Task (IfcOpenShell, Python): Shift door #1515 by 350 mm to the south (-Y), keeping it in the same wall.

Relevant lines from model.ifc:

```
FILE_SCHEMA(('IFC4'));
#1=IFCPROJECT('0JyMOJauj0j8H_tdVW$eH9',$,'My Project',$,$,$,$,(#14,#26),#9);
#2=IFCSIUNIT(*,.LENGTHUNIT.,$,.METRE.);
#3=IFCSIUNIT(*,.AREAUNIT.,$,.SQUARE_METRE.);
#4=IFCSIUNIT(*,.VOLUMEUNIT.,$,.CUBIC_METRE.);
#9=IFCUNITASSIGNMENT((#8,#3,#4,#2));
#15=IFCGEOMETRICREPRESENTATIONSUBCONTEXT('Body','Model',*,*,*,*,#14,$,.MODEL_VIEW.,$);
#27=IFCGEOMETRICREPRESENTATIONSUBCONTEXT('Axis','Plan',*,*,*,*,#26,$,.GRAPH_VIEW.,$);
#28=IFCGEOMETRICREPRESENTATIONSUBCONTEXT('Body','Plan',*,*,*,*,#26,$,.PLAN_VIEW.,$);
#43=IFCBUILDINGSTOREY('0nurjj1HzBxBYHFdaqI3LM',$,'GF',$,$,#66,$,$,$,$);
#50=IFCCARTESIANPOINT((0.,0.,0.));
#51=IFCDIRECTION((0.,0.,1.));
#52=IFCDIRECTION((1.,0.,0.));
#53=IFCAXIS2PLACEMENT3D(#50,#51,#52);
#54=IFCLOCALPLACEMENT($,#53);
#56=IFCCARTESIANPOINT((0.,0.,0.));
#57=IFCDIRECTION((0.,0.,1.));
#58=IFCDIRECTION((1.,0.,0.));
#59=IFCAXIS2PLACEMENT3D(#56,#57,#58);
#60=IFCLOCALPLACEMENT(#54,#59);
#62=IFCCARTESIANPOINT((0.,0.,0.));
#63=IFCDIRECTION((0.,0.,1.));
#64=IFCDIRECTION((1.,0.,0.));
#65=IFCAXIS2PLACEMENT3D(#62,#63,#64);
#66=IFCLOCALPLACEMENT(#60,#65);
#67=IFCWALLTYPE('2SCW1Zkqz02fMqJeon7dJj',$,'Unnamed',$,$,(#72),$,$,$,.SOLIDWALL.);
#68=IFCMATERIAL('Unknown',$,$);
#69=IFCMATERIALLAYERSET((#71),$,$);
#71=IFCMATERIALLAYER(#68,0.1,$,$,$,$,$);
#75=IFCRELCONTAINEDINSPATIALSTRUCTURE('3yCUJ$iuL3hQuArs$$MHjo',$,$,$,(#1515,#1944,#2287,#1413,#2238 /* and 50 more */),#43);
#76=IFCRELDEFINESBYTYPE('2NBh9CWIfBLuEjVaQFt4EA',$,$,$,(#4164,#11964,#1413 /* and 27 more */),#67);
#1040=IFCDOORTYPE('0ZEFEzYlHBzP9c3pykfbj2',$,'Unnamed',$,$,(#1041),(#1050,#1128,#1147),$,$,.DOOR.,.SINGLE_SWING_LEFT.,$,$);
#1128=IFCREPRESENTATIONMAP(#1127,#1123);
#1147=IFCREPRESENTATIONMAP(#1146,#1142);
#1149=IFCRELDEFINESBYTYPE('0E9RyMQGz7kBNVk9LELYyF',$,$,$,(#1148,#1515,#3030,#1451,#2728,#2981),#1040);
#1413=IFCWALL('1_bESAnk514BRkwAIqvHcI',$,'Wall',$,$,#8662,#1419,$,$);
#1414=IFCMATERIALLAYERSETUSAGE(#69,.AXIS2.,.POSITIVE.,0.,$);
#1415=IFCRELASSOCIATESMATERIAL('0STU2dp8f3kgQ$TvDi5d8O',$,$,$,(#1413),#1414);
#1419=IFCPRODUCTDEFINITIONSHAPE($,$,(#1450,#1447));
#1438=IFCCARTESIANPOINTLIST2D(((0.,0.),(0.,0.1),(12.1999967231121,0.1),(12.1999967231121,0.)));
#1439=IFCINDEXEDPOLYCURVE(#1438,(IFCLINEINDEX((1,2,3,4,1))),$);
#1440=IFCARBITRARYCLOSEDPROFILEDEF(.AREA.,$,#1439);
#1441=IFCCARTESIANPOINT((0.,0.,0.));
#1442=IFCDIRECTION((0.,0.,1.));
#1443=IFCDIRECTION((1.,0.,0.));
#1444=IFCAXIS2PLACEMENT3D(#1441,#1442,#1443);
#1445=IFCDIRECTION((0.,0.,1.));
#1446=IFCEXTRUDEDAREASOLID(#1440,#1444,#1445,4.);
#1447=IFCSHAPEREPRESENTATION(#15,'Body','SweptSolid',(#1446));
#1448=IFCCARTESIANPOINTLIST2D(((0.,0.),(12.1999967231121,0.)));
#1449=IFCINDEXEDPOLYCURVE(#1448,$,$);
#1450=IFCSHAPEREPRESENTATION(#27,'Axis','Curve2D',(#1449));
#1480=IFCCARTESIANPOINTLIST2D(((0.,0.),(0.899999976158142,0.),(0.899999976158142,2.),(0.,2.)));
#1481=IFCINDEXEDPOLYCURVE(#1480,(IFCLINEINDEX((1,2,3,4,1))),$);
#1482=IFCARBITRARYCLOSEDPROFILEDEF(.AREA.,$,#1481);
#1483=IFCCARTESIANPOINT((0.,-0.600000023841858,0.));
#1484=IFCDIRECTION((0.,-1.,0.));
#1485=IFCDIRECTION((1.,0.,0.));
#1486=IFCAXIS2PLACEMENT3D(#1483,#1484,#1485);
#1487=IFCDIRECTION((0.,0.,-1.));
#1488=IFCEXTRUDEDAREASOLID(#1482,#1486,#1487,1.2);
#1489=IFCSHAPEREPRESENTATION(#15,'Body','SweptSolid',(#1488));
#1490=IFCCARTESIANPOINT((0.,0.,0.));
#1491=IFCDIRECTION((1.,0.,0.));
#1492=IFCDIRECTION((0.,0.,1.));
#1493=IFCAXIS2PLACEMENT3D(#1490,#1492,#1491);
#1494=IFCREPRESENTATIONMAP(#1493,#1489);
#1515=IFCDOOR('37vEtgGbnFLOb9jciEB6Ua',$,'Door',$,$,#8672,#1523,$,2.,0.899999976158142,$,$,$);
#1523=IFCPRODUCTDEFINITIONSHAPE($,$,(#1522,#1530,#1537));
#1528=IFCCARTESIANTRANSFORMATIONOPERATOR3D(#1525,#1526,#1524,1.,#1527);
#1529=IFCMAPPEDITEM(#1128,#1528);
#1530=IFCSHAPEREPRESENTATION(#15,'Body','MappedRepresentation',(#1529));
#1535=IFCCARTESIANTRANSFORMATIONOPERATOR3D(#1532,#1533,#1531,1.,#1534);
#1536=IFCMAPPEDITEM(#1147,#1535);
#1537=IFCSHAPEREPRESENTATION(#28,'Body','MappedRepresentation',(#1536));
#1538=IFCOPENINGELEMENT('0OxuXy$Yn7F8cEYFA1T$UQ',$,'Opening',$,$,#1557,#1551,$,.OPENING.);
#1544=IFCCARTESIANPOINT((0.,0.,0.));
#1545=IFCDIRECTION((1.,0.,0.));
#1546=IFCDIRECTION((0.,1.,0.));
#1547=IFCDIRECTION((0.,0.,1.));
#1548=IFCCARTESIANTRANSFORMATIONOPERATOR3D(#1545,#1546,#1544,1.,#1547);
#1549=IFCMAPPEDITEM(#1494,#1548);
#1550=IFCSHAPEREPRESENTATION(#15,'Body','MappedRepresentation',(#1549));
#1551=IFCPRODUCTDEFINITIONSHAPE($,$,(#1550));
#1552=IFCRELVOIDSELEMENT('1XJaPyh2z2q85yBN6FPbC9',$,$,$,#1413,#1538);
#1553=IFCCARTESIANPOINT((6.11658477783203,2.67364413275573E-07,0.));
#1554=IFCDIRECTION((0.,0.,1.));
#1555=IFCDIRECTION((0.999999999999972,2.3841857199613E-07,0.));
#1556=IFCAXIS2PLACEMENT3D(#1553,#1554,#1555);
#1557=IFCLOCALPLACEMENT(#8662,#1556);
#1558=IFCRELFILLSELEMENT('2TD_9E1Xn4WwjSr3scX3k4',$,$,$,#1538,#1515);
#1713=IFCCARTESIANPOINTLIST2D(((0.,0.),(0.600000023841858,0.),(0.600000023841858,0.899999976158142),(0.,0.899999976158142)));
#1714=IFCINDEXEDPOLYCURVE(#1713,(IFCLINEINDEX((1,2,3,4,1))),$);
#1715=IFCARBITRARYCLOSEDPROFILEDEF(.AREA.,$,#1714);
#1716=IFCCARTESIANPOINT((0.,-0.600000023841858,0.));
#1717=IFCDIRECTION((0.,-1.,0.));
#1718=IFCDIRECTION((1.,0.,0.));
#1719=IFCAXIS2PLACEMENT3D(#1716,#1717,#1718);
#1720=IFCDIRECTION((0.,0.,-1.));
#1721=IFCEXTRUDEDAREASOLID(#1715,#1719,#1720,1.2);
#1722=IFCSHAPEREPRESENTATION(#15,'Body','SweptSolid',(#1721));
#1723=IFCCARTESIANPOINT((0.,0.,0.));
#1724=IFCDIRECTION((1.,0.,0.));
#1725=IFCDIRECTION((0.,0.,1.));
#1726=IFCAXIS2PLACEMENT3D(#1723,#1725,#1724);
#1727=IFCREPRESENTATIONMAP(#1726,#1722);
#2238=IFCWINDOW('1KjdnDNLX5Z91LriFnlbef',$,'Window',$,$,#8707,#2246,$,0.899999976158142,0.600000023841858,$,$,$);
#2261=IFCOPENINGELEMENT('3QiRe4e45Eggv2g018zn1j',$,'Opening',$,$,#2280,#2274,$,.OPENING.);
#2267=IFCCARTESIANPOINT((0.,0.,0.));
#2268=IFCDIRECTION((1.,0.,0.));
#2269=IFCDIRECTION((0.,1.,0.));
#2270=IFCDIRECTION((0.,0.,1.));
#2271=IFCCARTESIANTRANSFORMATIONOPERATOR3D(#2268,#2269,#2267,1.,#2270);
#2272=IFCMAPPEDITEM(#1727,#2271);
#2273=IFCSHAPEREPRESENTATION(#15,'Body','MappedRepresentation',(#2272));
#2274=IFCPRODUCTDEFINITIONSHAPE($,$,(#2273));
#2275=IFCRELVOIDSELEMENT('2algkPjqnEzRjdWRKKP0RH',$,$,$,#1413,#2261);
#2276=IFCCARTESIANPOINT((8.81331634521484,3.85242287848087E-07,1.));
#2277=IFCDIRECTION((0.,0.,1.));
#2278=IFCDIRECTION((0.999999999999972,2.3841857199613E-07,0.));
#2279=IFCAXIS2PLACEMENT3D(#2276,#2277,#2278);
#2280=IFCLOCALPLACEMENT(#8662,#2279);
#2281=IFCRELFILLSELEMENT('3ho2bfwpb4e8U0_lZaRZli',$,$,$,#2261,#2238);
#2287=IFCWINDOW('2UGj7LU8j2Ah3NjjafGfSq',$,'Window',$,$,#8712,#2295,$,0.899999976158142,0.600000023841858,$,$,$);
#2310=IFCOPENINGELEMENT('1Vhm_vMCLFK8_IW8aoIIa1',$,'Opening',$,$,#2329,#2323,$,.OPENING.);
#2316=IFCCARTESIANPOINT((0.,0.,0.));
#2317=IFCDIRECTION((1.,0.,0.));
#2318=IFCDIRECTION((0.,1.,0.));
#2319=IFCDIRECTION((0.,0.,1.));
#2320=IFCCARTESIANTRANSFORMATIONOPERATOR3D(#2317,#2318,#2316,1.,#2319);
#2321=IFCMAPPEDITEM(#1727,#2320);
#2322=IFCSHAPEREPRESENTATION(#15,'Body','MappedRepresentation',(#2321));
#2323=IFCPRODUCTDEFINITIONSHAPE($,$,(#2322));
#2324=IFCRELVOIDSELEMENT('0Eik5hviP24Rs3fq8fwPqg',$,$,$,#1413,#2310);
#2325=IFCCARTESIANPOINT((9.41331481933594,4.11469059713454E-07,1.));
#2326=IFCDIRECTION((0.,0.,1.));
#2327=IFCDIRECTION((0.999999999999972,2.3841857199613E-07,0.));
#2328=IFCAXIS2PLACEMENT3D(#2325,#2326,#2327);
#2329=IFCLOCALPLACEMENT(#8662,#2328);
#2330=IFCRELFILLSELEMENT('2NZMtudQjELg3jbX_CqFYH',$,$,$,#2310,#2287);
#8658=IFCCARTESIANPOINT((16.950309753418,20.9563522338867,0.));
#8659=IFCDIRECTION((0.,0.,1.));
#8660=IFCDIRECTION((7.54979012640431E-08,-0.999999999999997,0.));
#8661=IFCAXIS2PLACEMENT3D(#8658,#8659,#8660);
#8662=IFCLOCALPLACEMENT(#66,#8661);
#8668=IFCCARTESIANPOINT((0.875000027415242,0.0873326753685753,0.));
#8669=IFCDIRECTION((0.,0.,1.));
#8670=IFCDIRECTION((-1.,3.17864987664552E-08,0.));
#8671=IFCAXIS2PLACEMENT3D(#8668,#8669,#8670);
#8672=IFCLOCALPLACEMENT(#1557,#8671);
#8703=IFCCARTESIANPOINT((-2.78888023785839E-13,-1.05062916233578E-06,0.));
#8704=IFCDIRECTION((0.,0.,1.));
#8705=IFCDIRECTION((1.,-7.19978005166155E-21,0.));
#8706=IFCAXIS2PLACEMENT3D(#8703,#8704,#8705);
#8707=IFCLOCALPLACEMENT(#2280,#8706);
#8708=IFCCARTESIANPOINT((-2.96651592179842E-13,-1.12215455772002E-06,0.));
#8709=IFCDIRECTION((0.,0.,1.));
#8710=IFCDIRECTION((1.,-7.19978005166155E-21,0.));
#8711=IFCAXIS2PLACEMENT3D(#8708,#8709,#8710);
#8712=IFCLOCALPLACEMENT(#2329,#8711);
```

```python
import ifcopenshell
import ifcopenshell.api.geometry
import ifcopenshell.util.placement
import ifcopenshell.util.unit

model = ifcopenshell.open("model.ifc")
unit_scale = ifcopenshell.util.unit.calculate_unit_scale(model)

door = model.by_guid("37vEtgGbnFLOb9jciEB6Ua")
opening = door.FillsVoids[0].RelatingOpeningElement
wall = opening.VoidsElements[0].RelatingBuildingElement

wall_matrix = ifcopenshell.util.placement.get_local_placement(wall.ObjectPlacement)
shift = wall_matrix[:3, 0] * 0.35 / unit_scale
before = ifcopenshell.util.placement.get_local_placement(door.ObjectPlacement)[:3, 3].copy()

# The door is placed relative to its opening, so it follows when the opening moves.
matrix = ifcopenshell.util.placement.get_local_placement(opening.ObjectPlacement)
matrix[:3, 3] += shift
ifcopenshell.api.geometry.edit_object_placement(
    model, product=opening, matrix=matrix, is_si=False, should_transform_children=True
)

after = ifcopenshell.util.placement.get_local_placement(door.ObjectPlacement)[:3, 3]
print("door moved by", (after - before).round(3) + 0.0)

model.write("model_rev.ifc")
```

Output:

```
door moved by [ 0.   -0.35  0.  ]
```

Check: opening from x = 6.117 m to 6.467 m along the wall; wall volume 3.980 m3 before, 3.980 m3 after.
